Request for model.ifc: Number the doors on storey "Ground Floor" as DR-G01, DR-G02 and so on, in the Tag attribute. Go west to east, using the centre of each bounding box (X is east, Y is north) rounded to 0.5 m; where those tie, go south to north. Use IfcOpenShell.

First a look at what the model holds.

```python
import ifcopenshell
import ifcopenshell.util.element
import ifcopenshell.util.placement

model = ifcopenshell.open("model.ifc")
print(model.schema)
storey = next(s for s in model.by_type("IfcBuildingStorey") if s.Name == "Ground Floor")
doors = [e for e in ifcopenshell.util.element.get_decomposition(storey) if e.is_a("IfcDoor")]
for e in sorted(doors, key=lambda e: e.id()):
    origin = ifcopenshell.util.placement.get_local_placement(e.ObjectPlacement)[:3, 3]
    print(e.id(), e.Tag, e.Name, origin.round(2) + 0.0, sep=" | ")
```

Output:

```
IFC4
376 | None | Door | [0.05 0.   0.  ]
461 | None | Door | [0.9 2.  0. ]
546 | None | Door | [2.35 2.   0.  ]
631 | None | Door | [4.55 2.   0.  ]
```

```python
import ifcopenshell
import ifcopenshell.geom
import ifcopenshell.util.element
import ifcopenshell.util.shape

model = ifcopenshell.open("model.ifc")
settings = ifcopenshell.geom.settings()
settings.set("use-world-coords", True)


def centre(element):
    shape = ifcopenshell.geom.create_shape(settings, element)
    return ifcopenshell.util.shape.get_bbox_centroid(shape.geometry)


storey = next(s for s in model.by_type("IfcBuildingStorey") if s.Name == "Ground Floor")
doors = [e for e in ifcopenshell.util.element.get_decomposition(storey) if e.is_a("IfcDoor")]

# Insertion points can sit at a corner or the storey origin, so sort by the geometry (in metres).
centres = {e: centre(e) for e in doors}
doors.sort(key=lambda e: (round(centres[e][0] / 0.5), centres[e][1]))

for i, e in enumerate(doors, start=1):
    number = f"DR-G{i:02d}"
    e.Tag = number
    print(e.id(), number)

model.write("model_v2.ifc")
```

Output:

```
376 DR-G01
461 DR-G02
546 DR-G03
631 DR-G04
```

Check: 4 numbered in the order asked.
